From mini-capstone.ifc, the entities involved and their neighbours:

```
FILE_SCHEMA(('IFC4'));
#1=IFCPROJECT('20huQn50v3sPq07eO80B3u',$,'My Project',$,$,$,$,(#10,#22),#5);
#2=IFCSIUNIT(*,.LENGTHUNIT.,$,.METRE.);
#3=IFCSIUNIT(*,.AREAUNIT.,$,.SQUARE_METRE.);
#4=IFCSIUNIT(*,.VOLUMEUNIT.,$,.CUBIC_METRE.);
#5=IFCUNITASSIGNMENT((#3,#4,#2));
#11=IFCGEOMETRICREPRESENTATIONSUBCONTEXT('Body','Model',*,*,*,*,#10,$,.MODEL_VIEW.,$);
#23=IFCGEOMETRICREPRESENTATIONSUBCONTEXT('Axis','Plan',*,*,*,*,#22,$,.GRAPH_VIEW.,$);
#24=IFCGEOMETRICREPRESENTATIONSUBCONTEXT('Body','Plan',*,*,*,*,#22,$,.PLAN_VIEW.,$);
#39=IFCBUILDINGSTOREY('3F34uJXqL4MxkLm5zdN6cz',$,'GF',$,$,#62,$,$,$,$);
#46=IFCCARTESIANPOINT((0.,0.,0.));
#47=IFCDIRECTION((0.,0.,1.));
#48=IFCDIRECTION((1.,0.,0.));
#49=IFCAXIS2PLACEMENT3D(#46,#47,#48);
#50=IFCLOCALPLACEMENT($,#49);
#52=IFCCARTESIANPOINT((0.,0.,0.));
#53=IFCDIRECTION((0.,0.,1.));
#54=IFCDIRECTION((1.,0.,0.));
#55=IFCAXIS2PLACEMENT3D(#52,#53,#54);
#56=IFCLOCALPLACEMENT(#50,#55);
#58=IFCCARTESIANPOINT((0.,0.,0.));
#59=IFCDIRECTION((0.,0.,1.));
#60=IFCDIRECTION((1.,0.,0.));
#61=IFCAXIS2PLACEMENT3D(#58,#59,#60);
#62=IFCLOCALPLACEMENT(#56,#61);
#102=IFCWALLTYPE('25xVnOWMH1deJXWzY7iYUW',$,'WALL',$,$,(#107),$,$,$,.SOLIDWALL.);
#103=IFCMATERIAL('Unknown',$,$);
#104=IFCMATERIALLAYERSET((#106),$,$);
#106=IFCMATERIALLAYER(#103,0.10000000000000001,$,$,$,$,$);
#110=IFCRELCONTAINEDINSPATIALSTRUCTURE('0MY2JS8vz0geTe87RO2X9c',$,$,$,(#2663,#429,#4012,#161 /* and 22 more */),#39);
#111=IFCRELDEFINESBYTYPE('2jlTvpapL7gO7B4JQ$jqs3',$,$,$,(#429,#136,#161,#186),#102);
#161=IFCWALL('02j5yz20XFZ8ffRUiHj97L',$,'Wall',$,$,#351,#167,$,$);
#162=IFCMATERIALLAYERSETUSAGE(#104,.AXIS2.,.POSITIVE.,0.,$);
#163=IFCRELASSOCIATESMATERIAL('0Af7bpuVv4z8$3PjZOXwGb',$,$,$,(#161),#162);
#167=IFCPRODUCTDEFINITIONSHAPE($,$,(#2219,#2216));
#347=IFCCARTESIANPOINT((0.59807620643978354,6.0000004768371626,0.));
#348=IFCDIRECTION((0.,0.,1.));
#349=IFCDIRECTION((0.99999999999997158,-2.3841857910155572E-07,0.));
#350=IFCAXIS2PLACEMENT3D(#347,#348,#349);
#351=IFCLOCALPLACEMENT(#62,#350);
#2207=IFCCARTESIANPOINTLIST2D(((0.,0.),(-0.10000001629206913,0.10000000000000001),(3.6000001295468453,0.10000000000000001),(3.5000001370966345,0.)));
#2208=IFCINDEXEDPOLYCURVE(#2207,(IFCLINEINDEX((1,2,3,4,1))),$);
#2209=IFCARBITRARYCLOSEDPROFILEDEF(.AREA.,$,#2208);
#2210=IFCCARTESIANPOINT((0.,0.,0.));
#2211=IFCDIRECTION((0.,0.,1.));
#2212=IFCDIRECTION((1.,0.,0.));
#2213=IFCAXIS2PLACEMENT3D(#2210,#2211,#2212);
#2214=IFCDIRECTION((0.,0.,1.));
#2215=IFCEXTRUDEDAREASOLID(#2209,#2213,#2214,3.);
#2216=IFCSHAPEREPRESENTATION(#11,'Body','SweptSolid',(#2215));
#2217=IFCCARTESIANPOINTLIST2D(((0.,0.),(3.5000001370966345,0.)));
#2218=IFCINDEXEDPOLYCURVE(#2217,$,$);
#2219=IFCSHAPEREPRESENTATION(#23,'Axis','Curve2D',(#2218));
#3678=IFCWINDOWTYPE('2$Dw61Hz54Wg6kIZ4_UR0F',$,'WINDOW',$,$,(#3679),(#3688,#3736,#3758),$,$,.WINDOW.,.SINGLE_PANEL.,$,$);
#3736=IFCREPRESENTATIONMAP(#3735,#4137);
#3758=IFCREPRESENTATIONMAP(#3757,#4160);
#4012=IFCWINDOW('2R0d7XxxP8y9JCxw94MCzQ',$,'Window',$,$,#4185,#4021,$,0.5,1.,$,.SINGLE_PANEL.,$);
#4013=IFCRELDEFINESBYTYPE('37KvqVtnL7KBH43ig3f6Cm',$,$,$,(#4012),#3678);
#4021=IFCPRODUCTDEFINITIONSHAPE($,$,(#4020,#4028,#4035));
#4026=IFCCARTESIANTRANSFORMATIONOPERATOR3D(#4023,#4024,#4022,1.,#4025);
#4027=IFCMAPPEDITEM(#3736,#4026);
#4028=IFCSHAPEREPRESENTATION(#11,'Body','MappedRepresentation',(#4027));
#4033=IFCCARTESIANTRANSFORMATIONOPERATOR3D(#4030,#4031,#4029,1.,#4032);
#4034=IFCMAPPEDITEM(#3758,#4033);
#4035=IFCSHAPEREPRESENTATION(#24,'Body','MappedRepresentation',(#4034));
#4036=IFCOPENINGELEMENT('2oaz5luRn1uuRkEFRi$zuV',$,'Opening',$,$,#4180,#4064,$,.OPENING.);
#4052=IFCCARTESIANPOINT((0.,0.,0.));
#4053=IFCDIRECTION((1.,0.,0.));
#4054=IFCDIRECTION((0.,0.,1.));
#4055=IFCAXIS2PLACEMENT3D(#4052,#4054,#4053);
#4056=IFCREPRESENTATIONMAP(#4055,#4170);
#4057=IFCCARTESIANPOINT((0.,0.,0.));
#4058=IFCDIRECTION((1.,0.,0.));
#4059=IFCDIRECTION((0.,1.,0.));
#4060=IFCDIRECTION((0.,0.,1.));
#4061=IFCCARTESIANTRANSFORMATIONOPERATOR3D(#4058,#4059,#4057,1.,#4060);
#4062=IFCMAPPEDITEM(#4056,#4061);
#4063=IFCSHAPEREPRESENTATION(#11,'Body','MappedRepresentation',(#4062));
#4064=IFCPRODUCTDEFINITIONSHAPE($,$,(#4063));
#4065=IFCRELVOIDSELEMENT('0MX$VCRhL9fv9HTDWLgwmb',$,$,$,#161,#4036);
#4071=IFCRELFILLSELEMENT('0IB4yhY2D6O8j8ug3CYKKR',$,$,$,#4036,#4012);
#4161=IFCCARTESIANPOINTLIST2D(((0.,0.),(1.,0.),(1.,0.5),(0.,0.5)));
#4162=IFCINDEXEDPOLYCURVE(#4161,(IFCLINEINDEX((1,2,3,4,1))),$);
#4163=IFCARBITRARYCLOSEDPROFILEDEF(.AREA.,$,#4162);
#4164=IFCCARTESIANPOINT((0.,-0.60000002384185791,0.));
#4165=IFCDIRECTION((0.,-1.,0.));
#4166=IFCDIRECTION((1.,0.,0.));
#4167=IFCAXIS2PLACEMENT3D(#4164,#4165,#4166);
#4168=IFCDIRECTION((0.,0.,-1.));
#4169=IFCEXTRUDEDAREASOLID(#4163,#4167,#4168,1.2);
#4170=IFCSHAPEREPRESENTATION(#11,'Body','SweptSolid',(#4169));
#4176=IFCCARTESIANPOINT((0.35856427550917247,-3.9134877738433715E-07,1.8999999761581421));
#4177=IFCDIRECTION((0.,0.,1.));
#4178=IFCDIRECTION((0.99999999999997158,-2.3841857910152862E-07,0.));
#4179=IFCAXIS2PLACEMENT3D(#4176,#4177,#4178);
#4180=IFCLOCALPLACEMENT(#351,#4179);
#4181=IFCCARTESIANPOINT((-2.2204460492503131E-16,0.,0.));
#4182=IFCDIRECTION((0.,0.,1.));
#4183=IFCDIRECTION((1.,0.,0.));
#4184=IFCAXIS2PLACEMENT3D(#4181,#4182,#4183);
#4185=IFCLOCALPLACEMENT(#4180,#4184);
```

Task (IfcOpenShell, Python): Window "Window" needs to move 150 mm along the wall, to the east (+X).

```python
import ifcopenshell
import ifcopenshell.api.geometry
import ifcopenshell.util.placement
import ifcopenshell.util.unit

model = ifcopenshell.open("mini-capstone.ifc")
unit_scale = ifcopenshell.util.unit.calculate_unit_scale(model)

window = model.by_guid("2R0d7XxxP8y9JCxw94MCzQ")
opening = window.FillsVoids[0].RelatingOpeningElement
wall = opening.VoidsElements[0].RelatingBuildingElement

wall_matrix = ifcopenshell.util.placement.get_local_placement(wall.ObjectPlacement)
shift = wall_matrix[:3, 0] * 0.15 / unit_scale
before = ifcopenshell.util.placement.get_local_placement(window.ObjectPlacement)[:3, 3].copy()

# The window is placed relative to its opening, so it follows when the opening moves.
matrix = ifcopenshell.util.placement.get_local_placement(opening.ObjectPlacement)
matrix[:3, 3] += shift
ifcopenshell.api.geometry.edit_object_placement(
    model, product=opening, matrix=matrix, is_si=False, should_transform_children=True
)

after = ifcopenshell.util.placement.get_local_placement(window.ObjectPlacement)[:3, 3]
print("window moved by", (after - before).round(3) + 0.0)

model.write("mini-capstone_rev.ifc")
```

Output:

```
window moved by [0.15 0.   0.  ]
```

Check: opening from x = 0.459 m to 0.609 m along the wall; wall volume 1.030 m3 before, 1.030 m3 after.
